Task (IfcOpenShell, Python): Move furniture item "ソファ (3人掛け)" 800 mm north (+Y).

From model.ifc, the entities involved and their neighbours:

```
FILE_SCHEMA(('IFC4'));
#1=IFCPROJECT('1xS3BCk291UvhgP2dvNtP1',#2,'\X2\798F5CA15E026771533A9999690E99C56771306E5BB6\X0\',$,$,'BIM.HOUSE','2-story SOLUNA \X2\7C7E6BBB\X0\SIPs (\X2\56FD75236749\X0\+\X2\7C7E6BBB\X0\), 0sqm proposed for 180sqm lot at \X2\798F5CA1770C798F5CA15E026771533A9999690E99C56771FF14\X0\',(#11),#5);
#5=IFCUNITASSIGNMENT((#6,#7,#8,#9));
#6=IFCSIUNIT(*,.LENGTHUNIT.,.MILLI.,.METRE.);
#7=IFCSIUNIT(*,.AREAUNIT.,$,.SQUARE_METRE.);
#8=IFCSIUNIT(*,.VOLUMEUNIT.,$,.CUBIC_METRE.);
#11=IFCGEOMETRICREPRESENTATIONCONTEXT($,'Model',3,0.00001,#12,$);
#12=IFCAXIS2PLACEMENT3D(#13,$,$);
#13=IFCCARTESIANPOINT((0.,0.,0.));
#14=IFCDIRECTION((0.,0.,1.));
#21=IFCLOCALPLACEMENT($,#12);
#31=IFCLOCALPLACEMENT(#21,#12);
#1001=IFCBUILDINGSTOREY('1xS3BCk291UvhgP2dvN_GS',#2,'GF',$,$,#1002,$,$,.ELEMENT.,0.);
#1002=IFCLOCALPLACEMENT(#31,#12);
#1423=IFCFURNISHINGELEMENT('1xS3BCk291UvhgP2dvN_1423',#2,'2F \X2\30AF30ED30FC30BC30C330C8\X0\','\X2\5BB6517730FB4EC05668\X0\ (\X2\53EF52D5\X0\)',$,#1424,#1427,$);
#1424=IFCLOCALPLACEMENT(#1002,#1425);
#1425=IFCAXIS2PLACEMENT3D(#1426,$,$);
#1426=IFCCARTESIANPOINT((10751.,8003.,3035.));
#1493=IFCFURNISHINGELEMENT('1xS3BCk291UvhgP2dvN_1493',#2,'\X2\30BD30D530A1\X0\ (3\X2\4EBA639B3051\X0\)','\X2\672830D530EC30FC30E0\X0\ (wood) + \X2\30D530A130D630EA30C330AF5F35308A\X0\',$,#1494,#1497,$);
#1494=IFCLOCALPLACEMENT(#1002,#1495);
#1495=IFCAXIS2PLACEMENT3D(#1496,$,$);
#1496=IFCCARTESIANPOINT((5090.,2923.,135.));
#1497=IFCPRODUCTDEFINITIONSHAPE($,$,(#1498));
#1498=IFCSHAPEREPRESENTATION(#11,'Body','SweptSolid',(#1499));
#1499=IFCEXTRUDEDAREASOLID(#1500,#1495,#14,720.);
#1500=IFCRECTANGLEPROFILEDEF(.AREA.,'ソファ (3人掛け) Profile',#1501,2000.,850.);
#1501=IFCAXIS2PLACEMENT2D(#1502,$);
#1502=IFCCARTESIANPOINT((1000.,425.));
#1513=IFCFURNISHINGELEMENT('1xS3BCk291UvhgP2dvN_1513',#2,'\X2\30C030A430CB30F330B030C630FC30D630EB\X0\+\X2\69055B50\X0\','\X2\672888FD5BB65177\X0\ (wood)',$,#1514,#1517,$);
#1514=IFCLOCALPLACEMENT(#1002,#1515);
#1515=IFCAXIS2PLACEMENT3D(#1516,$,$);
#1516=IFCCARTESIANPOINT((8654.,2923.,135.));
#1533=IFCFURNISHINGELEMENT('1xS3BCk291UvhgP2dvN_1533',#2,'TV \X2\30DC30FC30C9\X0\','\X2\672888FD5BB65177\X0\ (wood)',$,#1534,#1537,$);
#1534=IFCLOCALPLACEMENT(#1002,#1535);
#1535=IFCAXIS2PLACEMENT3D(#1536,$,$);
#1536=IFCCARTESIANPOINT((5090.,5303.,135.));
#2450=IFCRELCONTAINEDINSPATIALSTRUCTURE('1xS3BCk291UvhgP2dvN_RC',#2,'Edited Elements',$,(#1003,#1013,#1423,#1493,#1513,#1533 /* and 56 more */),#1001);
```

```python
import ifcopenshell
import ifcopenshell.api.geometry
import ifcopenshell.util.placement
import ifcopenshell.util.unit

model = ifcopenshell.open("model.ifc")
unit_scale = ifcopenshell.util.unit.calculate_unit_scale(model)

item = model.by_guid("1xS3BCk291UvhgP2dvN_1493")
matrix = ifcopenshell.util.placement.get_local_placement(item.ObjectPlacement)
matrix[1, 3] += 0.8 / unit_scale
ifcopenshell.api.geometry.edit_object_placement(model, product=item, matrix=matrix, is_si=False)

print(ifcopenshell.util.placement.get_local_placement(item.ObjectPlacement).round(3) + 0.0)

model.write("model_edited.ifc")
```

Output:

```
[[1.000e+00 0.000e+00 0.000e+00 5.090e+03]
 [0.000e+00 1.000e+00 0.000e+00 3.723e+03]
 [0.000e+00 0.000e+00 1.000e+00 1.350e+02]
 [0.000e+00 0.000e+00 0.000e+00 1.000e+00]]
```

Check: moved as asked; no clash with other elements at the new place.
